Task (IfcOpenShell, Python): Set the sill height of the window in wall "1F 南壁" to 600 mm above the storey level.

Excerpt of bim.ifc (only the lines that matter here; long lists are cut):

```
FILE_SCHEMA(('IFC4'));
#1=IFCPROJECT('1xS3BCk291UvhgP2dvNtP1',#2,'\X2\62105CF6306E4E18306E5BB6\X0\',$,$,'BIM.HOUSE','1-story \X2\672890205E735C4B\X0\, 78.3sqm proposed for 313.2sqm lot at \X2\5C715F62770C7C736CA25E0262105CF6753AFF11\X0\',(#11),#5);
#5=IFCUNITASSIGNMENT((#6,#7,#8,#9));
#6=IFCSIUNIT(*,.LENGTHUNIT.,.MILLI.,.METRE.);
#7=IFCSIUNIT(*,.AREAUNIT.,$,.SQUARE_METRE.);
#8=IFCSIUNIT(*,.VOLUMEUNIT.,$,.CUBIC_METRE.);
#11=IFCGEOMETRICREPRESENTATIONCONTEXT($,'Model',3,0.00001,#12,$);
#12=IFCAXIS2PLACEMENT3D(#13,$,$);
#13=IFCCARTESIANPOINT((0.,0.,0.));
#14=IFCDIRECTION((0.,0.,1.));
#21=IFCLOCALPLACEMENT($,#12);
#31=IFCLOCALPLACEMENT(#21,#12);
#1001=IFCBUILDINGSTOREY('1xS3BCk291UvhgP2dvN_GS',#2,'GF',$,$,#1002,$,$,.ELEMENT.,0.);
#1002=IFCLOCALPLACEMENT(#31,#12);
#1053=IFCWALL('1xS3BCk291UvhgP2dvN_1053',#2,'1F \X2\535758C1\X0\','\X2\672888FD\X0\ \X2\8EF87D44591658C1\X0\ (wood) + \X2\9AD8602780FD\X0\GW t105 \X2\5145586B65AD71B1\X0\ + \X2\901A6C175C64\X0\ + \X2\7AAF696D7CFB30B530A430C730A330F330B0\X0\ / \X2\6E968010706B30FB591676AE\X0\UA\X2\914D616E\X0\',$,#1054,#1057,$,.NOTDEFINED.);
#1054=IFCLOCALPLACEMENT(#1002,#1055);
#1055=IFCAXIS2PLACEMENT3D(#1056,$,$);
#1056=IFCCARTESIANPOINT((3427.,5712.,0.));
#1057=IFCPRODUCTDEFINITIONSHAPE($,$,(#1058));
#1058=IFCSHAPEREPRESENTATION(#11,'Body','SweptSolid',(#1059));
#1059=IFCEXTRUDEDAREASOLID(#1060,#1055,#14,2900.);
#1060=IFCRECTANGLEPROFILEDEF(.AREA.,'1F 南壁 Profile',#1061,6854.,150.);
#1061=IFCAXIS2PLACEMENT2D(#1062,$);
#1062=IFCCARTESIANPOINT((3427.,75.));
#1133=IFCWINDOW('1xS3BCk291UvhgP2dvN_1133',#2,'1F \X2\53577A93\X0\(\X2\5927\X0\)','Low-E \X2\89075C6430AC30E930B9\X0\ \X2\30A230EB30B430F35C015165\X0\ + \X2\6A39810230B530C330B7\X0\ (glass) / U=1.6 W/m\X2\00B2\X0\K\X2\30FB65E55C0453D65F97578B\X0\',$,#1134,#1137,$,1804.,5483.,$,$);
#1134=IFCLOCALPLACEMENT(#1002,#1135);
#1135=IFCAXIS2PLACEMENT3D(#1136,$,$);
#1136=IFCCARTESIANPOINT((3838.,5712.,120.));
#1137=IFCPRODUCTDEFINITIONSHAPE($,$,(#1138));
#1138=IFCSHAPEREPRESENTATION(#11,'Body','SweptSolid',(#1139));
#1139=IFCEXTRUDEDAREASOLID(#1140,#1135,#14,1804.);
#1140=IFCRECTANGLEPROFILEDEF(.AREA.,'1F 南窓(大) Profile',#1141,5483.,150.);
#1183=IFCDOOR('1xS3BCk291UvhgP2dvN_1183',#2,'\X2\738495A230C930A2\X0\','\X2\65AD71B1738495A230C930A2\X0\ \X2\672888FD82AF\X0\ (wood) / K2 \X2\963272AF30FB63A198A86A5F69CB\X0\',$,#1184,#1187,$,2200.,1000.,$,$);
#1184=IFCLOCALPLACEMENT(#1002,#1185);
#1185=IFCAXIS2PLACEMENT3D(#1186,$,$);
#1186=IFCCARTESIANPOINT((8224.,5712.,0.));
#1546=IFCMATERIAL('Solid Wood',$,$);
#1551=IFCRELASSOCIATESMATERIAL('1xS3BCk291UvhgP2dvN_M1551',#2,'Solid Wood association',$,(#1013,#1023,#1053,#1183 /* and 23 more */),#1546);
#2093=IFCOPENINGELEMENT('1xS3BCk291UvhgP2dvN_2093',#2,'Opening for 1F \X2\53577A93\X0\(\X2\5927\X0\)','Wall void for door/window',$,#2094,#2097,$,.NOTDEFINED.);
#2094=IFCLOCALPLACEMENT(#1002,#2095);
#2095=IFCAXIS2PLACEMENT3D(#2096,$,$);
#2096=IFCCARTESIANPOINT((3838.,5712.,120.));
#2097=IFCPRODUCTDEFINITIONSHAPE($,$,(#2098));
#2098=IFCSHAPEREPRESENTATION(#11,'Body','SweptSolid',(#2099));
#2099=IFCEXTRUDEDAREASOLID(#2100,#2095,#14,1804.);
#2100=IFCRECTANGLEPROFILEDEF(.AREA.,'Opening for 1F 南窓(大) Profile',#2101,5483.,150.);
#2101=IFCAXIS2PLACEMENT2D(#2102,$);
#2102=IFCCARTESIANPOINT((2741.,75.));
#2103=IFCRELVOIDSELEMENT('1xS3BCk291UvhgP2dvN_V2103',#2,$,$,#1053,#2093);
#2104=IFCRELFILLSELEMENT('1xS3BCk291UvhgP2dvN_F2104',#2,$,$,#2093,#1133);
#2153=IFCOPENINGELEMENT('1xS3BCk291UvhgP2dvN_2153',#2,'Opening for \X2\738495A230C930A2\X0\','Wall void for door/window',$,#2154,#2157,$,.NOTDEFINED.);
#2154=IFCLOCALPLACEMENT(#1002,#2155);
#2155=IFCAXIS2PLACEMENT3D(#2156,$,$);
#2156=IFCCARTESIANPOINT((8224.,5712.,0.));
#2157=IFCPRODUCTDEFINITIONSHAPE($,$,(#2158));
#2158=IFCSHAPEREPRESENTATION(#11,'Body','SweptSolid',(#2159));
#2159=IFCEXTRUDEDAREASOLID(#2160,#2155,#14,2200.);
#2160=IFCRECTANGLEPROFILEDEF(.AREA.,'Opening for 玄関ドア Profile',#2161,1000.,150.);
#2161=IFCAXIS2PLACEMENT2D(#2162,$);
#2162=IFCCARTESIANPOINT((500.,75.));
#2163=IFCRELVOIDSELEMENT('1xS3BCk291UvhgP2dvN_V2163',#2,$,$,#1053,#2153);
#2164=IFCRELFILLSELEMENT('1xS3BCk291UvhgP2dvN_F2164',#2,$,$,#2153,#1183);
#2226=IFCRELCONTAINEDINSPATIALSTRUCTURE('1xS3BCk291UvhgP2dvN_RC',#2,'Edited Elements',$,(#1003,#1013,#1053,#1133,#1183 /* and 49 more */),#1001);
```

```python
import numpy as np
import ifcopenshell
import ifcopenshell.api.geometry
import ifcopenshell.geom
import ifcopenshell.util.element
import ifcopenshell.util.placement
import ifcopenshell.util.shape
import ifcopenshell.util.unit

model = ifcopenshell.open("bim.ifc")
unit_scale = ifcopenshell.util.unit.calculate_unit_scale(model)

window = model.by_guid("1xS3BCk291UvhgP2dvN_1133")
opening = window.FillsVoids[0].RelatingOpeningElement
storey = ifcopenshell.util.element.get_container(window, ifc_class="IfcBuildingStorey")
level = ifcopenshell.util.placement.get_local_placement(storey.ObjectPlacement)[2, 3]

# The opening's origin need not be at the sill, so measure its lowest point.
shape = ifcopenshell.geom.create_shape(ifcopenshell.geom.settings(), opening)
bottom = ifcopenshell.util.shape.get_shape_bottom_elevation(shape, shape.geometry) / unit_scale
dz = level + 0.6 / unit_scale - bottom

shift = np.array([0.0, 0.0, dz])
# The window is not placed relative to its opening, so move both.
for product in (opening, window):
    matrix = ifcopenshell.util.placement.get_local_placement(product.ObjectPlacement)
    matrix[:3, 3] += shift
    ifcopenshell.api.geometry.edit_object_placement(model, product=product, matrix=matrix, is_si=False)

print(f"moved by {dz * unit_scale:+.3f} m")

model.write("bim_edited.ifc")
```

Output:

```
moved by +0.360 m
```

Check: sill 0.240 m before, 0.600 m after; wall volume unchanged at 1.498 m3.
